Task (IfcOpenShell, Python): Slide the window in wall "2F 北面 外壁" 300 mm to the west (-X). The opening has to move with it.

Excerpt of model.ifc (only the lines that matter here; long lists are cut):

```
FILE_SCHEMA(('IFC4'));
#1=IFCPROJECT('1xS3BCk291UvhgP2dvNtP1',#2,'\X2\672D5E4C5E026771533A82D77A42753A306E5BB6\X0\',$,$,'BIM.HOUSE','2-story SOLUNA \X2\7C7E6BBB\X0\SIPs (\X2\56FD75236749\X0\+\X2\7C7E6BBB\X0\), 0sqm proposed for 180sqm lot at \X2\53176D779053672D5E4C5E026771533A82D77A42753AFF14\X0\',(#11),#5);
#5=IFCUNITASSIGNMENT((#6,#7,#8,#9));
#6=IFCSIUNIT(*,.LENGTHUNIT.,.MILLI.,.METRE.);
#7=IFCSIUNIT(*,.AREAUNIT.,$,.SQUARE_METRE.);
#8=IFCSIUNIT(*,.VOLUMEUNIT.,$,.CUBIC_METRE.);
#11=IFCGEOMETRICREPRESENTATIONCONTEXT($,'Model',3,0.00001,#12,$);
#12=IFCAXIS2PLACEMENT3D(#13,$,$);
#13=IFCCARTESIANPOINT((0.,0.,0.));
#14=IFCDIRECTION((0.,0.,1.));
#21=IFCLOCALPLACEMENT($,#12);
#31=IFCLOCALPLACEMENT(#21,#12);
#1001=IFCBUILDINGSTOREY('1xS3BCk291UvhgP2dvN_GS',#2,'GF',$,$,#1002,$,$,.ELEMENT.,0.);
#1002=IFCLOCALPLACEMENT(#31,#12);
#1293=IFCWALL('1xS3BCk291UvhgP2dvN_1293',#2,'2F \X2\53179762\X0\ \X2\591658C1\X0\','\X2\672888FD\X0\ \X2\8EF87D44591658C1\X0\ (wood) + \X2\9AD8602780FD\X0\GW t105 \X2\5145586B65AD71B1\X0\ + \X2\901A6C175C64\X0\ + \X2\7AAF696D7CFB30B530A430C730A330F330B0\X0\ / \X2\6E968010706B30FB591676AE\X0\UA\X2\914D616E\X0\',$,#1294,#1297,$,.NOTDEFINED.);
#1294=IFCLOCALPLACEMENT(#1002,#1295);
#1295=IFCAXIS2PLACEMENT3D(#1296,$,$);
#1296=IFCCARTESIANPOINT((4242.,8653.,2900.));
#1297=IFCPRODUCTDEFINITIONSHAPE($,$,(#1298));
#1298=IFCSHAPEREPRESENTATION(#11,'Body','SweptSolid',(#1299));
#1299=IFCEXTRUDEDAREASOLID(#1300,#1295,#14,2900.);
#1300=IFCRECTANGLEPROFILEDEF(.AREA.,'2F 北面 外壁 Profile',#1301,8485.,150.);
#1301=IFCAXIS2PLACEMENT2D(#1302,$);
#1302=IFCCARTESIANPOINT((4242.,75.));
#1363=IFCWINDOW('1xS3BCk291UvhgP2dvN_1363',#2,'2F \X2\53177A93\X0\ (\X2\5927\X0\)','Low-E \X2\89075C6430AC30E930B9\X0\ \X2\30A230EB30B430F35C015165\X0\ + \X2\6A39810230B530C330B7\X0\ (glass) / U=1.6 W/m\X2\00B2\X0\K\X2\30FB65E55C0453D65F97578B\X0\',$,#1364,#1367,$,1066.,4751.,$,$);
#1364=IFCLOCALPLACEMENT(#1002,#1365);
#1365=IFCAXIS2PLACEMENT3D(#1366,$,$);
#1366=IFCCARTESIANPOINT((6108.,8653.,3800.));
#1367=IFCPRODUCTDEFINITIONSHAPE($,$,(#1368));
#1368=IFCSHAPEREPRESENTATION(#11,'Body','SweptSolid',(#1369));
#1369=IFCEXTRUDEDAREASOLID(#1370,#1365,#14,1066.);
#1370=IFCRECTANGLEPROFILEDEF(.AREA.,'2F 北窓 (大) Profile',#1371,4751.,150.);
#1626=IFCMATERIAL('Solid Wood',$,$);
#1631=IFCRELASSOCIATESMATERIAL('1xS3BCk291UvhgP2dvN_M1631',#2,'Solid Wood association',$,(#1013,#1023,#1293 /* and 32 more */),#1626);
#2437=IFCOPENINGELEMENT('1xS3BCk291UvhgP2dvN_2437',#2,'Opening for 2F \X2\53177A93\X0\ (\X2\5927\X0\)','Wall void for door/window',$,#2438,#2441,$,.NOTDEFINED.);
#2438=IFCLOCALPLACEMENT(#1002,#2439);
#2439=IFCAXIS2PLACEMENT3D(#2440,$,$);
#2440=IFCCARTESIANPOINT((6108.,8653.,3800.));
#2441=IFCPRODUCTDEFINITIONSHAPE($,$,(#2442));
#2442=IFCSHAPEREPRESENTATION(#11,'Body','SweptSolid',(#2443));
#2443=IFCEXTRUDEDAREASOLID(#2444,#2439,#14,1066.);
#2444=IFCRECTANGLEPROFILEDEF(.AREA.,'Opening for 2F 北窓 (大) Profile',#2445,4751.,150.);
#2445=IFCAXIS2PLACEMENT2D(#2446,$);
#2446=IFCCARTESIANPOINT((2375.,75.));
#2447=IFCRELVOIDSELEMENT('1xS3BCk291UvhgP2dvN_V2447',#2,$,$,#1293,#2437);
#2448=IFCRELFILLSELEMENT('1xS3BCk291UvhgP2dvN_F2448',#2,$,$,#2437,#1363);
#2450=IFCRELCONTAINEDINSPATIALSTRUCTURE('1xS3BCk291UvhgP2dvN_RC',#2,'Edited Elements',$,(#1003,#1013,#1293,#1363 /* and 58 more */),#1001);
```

```python
import ifcopenshell
import ifcopenshell.api.geometry
import ifcopenshell.util.placement
import ifcopenshell.util.unit

model = ifcopenshell.open("model.ifc")
unit_scale = ifcopenshell.util.unit.calculate_unit_scale(model)

window = model.by_guid("1xS3BCk291UvhgP2dvN_1363")
opening = window.FillsVoids[0].RelatingOpeningElement
wall = opening.VoidsElements[0].RelatingBuildingElement

wall_matrix = ifcopenshell.util.placement.get_local_placement(wall.ObjectPlacement)
shift = wall_matrix[:3, 0] * -0.3 / unit_scale
before = ifcopenshell.util.placement.get_local_placement(window.ObjectPlacement)[:3, 3].copy()

# The window is not placed relative to its opening, so move both.
for product in (opening, window):
    matrix = ifcopenshell.util.placement.get_local_placement(product.ObjectPlacement)
    matrix[:3, 3] += shift
    ifcopenshell.api.geometry.edit_object_placement(model, product=product, matrix=matrix, is_si=False)

after = ifcopenshell.util.placement.get_local_placement(window.ObjectPlacement)[:3, 3]
print("window moved by", (after - before).round(3) + 0.0)

model.write("model_v2.ifc")
```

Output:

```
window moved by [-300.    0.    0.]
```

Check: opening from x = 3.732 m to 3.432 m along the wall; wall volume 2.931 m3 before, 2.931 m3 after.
